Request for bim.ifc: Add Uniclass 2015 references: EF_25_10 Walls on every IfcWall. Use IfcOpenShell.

First a look at what the model holds.

```python
import ifcopenshell

model = ifcopenshell.open("bim.ifc")
print(model.schema)
print("classifications:", [c.Name for c in model.by_type("IfcClassification")])
for ifc_class in ("IfcDoor", "IfcRoof", "IfcStair", "IfcWall", "IfcWindow"):
    print(ifc_class, len(model.by_type(ifc_class)))
```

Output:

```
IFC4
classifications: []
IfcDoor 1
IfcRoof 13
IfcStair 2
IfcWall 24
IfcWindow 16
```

```python
import ifcopenshell
import ifcopenshell.api.classification

model = ifcopenshell.open("bim.ifc")

system = ifcopenshell.api.classification.add_classification(model, classification="Uniclass 2015")

codes = {
    "IfcWall": ("EF_25_10", "Walls"),
}
for ifc_class, (code, name) in codes.items():
    products = model.by_type(ifc_class)
    ifcopenshell.api.classification.add_reference(
        model, products=products, classification=system, identification=code, name=name
    )
    print(code, len(products))

model.write("bim_updated.ifc")
```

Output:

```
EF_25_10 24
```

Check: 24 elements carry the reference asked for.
